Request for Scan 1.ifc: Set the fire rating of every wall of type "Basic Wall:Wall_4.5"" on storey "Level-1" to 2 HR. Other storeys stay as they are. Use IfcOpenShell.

First a look at what the model holds.

```python
import ifcopenshell
import ifcopenshell.util.element

model = ifcopenshell.open("Scan 1.ifc")
print(model.schema)
storey = next(s for s in model.by_type("IfcBuildingStorey") if s.Name == "Level-1")
walls = [e for e in ifcopenshell.util.element.get_decomposition(storey) if e.is_a("IfcWall")]
seen = {}
for e in walls:
    element_type = ifcopenshell.util.element.get_type(e)
    key = (element_type.Name if element_type != e and element_type else None, ifcopenshell.util.element.get_pset(e, "Pset_WallCommon", "FireRating"))
    seen[key] = seen.get(key, 0) + 1
for (name, value), count in sorted(seen.items(), key=str):
    print(count, "x", name, "|", value)
```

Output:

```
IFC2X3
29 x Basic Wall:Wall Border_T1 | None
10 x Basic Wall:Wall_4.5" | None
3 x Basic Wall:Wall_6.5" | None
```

```python
import ifcopenshell
import ifcopenshell.api.pset
import ifcopenshell.util.element

model = ifcopenshell.open("Scan 1.ifc")

storey = next(s for s in model.by_type("IfcBuildingStorey") if s.Name == "Level-1")
walls = [e for e in ifcopenshell.util.element.get_decomposition(storey) if e.is_a("IfcWall")]

count = 0
for e in walls:
    element_type = ifcopenshell.util.element.get_type(e)
    if element_type in (None, e) or element_type.Name != 'Basic Wall:Wall_4.5"':
        continue
    # add_pset returns the element's existing set when there is one.
    pset = ifcopenshell.api.pset.add_pset(model, product=e, name="Pset_WallCommon")
    ifcopenshell.api.pset.edit_pset(model, pset=pset, properties={"FireRating": "2 HR"})
    count += 1

print(count, "walls updated")

model.write("Scan 1_edited.ifc")
```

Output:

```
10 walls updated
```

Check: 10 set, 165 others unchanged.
